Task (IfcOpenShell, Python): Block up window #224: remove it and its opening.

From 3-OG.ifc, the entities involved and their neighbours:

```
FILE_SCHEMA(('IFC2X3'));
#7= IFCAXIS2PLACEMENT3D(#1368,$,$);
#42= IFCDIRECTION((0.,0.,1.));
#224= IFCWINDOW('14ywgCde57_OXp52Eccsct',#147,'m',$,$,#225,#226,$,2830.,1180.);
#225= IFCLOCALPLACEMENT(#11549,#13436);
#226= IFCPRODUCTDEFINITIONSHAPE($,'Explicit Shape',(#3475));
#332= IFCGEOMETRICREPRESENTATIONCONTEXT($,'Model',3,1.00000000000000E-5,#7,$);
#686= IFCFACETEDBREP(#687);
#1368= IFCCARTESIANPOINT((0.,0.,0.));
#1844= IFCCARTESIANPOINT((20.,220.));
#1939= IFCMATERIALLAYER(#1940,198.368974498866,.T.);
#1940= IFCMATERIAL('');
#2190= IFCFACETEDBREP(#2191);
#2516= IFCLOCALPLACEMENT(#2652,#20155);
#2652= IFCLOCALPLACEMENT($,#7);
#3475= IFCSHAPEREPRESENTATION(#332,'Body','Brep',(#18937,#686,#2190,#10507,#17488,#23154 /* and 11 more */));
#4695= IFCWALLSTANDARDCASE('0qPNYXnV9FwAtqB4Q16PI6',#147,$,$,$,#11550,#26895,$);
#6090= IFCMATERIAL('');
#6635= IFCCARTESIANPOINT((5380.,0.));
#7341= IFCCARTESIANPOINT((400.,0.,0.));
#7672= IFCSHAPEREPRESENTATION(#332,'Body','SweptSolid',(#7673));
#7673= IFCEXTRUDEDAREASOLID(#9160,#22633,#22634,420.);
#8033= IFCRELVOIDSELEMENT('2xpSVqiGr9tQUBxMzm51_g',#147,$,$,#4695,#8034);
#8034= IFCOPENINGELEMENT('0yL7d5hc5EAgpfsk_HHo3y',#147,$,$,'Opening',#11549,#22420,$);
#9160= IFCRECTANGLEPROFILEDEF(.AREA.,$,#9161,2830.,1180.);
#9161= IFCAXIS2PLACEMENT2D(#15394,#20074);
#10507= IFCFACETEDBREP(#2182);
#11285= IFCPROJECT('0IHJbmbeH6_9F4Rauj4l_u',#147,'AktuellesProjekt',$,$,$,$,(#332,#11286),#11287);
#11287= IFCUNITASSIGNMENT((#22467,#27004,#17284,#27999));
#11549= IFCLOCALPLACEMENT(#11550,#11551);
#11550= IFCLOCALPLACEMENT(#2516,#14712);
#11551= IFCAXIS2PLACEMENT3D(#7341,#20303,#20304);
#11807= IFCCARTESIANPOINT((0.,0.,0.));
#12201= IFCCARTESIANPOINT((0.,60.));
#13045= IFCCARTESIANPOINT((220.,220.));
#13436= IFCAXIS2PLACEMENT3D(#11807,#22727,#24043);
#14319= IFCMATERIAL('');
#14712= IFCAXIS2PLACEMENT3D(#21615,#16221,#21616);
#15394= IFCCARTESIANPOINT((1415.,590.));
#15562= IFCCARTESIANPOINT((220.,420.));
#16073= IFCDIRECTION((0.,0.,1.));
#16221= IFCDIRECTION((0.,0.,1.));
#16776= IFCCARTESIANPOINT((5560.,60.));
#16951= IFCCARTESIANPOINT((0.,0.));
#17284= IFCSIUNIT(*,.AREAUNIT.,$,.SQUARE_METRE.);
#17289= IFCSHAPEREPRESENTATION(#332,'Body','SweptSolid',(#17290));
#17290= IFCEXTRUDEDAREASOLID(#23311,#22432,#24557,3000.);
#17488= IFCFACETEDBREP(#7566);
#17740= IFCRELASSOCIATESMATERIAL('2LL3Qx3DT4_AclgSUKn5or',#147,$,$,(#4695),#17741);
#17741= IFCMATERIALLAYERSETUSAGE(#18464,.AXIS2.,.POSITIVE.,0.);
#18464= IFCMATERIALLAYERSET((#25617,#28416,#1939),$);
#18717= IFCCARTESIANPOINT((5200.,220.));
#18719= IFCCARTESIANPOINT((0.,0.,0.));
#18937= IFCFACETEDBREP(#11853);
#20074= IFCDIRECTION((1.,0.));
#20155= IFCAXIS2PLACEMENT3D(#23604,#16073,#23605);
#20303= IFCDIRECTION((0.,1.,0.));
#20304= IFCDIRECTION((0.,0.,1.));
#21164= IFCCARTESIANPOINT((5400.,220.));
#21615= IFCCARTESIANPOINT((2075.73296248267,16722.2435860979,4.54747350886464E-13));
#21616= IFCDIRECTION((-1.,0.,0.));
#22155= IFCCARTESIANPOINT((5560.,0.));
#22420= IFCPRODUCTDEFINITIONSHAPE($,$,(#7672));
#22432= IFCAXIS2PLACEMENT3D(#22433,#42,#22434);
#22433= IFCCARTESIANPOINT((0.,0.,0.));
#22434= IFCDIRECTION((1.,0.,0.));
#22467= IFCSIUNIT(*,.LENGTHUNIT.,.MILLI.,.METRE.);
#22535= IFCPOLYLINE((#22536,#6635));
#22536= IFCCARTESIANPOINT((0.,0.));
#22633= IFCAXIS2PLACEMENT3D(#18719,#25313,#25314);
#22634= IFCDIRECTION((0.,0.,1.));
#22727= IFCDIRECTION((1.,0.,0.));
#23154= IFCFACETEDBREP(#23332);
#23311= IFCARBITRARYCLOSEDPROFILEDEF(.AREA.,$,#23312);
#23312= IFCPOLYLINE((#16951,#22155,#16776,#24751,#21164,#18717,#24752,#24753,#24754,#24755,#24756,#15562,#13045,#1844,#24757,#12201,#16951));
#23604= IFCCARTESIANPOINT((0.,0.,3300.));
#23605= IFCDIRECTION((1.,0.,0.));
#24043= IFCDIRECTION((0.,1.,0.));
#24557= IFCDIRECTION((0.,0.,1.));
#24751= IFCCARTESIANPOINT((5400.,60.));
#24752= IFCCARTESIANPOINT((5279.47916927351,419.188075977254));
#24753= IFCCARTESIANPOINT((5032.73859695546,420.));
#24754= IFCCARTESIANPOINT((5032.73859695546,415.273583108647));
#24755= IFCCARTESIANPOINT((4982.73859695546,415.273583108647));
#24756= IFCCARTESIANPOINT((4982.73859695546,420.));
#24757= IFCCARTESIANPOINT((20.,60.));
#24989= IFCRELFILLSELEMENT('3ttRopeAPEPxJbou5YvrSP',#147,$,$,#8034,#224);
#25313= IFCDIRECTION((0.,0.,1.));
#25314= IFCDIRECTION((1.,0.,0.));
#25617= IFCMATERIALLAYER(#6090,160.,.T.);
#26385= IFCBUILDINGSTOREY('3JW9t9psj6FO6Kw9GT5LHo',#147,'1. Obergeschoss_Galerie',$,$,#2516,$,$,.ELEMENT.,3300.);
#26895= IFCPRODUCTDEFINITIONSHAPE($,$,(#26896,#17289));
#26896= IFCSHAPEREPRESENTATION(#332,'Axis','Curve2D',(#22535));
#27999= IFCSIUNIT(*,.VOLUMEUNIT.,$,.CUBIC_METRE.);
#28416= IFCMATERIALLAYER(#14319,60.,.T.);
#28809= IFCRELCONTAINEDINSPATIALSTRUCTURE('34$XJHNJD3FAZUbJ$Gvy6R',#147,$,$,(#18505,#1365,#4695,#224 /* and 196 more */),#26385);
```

```python
import ifcopenshell
import ifcopenshell.api.feature
import ifcopenshell.api.root
import ifcopenshell.geom
import ifcopenshell.util.shape

model = ifcopenshell.open("3-OG.ifc")
settings = ifcopenshell.geom.settings()


def volume(element):
    """Net volume in cubic metres, openings subtracted."""
    shape = ifcopenshell.geom.create_shape(settings, element)
    return ifcopenshell.util.shape.get_volume(shape.geometry)


window = model.by_guid("14ywgCde57_OXp52Eccsct")
opening = window.FillsVoids[0].RelatingOpeningElement
wall = opening.VoidsElements[0].RelatingBuildingElement
before = volume(wall)

ifcopenshell.api.root.remove_product(model, product=window)
ifcopenshell.api.feature.remove_feature(model, feature=opening)

after = volume(wall)

print(f"wall volume {before:.3f} -> {after:.3f} m3")

model.write("3-OG_v2.ifc")
```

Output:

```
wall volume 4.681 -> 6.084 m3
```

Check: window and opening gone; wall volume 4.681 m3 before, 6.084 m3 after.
